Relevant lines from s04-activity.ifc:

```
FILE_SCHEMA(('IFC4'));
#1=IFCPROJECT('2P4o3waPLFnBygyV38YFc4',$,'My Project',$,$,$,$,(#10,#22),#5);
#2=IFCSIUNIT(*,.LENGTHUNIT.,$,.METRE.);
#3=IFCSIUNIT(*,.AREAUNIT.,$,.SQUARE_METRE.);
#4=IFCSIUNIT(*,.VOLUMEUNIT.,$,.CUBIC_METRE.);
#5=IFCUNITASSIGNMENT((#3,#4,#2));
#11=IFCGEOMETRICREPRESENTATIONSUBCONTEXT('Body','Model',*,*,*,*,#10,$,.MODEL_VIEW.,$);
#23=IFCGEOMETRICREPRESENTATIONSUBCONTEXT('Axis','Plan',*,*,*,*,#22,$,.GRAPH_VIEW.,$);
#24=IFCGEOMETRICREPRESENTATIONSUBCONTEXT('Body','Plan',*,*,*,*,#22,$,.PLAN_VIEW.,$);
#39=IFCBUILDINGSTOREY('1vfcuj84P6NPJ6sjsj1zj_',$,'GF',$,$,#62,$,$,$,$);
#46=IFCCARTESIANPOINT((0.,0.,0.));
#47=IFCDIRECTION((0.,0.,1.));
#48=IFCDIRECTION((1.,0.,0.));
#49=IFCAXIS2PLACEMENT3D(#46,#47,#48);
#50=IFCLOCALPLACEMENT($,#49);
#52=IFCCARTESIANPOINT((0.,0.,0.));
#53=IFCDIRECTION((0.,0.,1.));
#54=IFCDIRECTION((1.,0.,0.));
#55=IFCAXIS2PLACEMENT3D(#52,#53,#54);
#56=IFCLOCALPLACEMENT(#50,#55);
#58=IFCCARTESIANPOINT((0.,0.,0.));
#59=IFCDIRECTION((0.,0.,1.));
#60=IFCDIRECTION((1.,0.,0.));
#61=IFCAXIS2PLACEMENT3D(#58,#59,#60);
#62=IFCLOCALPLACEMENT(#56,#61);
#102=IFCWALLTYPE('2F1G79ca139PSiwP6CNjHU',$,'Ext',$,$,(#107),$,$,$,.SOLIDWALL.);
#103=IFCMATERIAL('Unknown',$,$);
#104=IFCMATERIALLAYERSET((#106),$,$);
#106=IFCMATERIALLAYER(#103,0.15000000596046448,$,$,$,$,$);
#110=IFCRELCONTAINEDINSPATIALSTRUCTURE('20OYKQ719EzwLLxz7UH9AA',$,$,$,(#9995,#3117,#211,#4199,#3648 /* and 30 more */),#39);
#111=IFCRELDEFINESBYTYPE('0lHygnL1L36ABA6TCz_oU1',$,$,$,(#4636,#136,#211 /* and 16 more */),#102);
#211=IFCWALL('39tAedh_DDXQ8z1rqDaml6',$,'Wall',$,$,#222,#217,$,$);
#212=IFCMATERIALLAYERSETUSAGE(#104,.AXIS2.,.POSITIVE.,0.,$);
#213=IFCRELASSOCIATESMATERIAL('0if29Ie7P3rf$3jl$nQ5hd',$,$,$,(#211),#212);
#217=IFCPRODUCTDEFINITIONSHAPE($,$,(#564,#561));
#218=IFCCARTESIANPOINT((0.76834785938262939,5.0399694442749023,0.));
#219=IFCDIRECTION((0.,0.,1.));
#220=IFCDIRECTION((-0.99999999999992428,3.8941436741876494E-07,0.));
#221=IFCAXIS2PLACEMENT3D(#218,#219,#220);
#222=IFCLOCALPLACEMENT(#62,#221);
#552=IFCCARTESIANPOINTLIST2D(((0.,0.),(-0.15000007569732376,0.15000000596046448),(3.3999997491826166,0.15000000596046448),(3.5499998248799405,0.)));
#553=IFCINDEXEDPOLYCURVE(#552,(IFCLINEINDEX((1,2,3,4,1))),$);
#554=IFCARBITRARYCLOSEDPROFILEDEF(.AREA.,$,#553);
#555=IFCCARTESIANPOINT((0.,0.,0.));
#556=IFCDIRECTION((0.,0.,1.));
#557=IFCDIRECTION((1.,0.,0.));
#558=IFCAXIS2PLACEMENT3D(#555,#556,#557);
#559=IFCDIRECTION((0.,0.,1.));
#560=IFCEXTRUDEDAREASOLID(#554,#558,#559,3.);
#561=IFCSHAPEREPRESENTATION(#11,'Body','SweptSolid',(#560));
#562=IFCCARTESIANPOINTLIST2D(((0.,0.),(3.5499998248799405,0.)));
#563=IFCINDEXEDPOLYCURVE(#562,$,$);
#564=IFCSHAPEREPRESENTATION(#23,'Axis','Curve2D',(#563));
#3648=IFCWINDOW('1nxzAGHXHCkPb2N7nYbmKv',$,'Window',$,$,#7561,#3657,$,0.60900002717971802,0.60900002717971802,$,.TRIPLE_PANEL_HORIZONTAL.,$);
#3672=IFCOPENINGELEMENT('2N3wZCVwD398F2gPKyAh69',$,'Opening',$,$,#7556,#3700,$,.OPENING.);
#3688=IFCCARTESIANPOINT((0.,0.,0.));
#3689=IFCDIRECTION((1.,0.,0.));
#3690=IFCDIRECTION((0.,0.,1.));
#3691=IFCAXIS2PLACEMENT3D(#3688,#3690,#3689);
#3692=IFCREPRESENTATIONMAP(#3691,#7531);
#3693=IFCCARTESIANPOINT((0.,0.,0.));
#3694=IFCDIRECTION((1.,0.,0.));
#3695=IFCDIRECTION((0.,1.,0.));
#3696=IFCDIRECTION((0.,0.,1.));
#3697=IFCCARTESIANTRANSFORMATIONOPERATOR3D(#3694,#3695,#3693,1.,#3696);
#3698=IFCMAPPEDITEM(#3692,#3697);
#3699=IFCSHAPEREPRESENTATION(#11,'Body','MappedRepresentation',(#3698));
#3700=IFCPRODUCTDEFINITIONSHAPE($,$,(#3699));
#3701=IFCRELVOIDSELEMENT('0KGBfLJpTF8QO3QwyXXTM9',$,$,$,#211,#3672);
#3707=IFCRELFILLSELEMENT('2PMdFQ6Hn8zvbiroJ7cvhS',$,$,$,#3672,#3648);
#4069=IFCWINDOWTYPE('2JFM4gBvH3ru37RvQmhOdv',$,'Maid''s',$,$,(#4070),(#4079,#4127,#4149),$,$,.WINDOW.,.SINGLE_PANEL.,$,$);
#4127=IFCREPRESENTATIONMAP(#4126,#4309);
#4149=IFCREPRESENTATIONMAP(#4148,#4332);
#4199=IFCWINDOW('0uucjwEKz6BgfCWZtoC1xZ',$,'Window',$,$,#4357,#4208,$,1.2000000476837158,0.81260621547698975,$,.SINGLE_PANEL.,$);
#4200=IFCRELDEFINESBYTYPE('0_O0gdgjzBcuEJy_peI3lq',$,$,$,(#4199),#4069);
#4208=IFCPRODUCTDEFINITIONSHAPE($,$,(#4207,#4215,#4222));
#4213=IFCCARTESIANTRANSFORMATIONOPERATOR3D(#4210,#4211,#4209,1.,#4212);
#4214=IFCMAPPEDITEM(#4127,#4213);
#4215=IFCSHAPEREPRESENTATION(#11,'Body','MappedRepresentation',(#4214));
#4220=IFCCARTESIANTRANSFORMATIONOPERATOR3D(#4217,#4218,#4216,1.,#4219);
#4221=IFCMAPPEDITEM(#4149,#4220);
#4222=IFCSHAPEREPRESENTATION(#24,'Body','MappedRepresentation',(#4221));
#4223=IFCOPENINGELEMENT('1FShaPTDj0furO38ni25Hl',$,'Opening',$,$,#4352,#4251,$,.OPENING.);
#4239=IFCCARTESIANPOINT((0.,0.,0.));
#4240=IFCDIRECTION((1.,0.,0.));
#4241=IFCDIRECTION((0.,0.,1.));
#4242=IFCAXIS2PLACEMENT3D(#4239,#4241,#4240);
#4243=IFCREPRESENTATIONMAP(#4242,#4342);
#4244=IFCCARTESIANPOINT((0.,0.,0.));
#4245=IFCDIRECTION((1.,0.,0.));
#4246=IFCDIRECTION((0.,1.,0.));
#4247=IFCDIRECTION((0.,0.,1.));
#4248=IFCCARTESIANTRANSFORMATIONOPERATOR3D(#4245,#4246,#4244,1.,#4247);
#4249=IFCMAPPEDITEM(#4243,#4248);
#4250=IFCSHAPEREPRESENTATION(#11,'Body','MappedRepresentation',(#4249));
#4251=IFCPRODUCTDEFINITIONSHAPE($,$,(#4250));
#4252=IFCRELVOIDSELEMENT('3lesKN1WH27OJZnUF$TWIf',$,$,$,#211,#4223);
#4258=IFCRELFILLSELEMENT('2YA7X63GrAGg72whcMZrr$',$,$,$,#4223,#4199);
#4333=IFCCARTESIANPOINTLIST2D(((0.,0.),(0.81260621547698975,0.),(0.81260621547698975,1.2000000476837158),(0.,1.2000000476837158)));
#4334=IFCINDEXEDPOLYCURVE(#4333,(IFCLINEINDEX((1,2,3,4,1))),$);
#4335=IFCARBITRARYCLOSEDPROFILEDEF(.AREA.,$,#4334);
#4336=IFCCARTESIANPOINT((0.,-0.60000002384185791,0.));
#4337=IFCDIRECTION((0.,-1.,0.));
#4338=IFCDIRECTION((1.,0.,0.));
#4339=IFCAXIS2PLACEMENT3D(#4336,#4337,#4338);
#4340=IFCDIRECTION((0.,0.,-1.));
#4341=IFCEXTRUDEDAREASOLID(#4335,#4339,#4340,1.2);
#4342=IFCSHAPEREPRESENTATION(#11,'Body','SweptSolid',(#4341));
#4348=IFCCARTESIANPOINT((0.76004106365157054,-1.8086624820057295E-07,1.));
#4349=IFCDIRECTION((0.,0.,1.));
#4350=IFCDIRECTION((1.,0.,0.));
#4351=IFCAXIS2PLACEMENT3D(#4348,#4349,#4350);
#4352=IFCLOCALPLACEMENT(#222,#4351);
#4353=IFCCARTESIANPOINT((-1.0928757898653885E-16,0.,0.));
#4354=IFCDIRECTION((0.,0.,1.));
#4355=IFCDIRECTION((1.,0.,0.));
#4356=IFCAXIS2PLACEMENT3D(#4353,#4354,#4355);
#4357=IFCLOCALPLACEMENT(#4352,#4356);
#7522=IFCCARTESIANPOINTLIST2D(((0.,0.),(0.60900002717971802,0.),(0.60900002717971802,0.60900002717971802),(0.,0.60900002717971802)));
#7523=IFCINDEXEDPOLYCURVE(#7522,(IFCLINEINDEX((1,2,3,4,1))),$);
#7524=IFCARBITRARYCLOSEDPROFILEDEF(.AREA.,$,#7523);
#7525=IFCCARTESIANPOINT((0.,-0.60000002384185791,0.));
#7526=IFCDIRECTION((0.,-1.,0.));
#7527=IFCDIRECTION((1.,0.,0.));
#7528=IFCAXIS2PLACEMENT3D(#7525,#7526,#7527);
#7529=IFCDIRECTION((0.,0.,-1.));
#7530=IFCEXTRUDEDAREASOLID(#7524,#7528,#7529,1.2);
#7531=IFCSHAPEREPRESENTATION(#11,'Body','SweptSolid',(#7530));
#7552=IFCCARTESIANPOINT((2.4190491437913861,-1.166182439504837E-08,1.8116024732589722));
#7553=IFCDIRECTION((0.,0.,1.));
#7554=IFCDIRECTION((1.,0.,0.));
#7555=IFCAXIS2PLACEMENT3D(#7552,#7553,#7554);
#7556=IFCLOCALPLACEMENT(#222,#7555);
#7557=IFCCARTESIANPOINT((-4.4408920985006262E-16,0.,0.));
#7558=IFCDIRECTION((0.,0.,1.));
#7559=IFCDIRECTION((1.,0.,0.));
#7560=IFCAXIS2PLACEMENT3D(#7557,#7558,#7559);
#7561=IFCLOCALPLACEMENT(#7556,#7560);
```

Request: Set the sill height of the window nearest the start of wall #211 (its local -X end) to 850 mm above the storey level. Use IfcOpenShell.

```python
import numpy as np
import ifcopenshell
import ifcopenshell.api.geometry
import ifcopenshell.geom
import ifcopenshell.util.element
import ifcopenshell.util.placement
import ifcopenshell.util.shape
import ifcopenshell.util.unit

model = ifcopenshell.open("s04-activity.ifc")
unit_scale = ifcopenshell.util.unit.calculate_unit_scale(model)

window = model.by_guid("0uucjwEKz6BgfCWZtoC1xZ")
opening = window.FillsVoids[0].RelatingOpeningElement
storey = ifcopenshell.util.element.get_container(window, ifc_class="IfcBuildingStorey")
level = ifcopenshell.util.placement.get_local_placement(storey.ObjectPlacement)[2, 3]

# The opening's origin need not be at the sill, so measure its lowest point.
shape = ifcopenshell.geom.create_shape(ifcopenshell.geom.settings(), opening)
bottom = ifcopenshell.util.shape.get_shape_bottom_elevation(shape, shape.geometry) / unit_scale
dz = level + 0.85 / unit_scale - bottom

shift = np.array([0.0, 0.0, dz])
# The window is placed relative to its opening, so it follows when the opening moves.
matrix = ifcopenshell.util.placement.get_local_placement(opening.ObjectPlacement)
matrix[:3, 3] += shift
ifcopenshell.api.geometry.edit_object_placement(
    model, product=opening, matrix=matrix, is_si=False, should_transform_children=True
)

print(f"moved by {dz * unit_scale:+.3f} m")

model.write("s04-activity_updated.ifc")
```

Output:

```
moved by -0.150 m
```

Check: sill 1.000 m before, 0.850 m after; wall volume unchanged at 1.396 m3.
